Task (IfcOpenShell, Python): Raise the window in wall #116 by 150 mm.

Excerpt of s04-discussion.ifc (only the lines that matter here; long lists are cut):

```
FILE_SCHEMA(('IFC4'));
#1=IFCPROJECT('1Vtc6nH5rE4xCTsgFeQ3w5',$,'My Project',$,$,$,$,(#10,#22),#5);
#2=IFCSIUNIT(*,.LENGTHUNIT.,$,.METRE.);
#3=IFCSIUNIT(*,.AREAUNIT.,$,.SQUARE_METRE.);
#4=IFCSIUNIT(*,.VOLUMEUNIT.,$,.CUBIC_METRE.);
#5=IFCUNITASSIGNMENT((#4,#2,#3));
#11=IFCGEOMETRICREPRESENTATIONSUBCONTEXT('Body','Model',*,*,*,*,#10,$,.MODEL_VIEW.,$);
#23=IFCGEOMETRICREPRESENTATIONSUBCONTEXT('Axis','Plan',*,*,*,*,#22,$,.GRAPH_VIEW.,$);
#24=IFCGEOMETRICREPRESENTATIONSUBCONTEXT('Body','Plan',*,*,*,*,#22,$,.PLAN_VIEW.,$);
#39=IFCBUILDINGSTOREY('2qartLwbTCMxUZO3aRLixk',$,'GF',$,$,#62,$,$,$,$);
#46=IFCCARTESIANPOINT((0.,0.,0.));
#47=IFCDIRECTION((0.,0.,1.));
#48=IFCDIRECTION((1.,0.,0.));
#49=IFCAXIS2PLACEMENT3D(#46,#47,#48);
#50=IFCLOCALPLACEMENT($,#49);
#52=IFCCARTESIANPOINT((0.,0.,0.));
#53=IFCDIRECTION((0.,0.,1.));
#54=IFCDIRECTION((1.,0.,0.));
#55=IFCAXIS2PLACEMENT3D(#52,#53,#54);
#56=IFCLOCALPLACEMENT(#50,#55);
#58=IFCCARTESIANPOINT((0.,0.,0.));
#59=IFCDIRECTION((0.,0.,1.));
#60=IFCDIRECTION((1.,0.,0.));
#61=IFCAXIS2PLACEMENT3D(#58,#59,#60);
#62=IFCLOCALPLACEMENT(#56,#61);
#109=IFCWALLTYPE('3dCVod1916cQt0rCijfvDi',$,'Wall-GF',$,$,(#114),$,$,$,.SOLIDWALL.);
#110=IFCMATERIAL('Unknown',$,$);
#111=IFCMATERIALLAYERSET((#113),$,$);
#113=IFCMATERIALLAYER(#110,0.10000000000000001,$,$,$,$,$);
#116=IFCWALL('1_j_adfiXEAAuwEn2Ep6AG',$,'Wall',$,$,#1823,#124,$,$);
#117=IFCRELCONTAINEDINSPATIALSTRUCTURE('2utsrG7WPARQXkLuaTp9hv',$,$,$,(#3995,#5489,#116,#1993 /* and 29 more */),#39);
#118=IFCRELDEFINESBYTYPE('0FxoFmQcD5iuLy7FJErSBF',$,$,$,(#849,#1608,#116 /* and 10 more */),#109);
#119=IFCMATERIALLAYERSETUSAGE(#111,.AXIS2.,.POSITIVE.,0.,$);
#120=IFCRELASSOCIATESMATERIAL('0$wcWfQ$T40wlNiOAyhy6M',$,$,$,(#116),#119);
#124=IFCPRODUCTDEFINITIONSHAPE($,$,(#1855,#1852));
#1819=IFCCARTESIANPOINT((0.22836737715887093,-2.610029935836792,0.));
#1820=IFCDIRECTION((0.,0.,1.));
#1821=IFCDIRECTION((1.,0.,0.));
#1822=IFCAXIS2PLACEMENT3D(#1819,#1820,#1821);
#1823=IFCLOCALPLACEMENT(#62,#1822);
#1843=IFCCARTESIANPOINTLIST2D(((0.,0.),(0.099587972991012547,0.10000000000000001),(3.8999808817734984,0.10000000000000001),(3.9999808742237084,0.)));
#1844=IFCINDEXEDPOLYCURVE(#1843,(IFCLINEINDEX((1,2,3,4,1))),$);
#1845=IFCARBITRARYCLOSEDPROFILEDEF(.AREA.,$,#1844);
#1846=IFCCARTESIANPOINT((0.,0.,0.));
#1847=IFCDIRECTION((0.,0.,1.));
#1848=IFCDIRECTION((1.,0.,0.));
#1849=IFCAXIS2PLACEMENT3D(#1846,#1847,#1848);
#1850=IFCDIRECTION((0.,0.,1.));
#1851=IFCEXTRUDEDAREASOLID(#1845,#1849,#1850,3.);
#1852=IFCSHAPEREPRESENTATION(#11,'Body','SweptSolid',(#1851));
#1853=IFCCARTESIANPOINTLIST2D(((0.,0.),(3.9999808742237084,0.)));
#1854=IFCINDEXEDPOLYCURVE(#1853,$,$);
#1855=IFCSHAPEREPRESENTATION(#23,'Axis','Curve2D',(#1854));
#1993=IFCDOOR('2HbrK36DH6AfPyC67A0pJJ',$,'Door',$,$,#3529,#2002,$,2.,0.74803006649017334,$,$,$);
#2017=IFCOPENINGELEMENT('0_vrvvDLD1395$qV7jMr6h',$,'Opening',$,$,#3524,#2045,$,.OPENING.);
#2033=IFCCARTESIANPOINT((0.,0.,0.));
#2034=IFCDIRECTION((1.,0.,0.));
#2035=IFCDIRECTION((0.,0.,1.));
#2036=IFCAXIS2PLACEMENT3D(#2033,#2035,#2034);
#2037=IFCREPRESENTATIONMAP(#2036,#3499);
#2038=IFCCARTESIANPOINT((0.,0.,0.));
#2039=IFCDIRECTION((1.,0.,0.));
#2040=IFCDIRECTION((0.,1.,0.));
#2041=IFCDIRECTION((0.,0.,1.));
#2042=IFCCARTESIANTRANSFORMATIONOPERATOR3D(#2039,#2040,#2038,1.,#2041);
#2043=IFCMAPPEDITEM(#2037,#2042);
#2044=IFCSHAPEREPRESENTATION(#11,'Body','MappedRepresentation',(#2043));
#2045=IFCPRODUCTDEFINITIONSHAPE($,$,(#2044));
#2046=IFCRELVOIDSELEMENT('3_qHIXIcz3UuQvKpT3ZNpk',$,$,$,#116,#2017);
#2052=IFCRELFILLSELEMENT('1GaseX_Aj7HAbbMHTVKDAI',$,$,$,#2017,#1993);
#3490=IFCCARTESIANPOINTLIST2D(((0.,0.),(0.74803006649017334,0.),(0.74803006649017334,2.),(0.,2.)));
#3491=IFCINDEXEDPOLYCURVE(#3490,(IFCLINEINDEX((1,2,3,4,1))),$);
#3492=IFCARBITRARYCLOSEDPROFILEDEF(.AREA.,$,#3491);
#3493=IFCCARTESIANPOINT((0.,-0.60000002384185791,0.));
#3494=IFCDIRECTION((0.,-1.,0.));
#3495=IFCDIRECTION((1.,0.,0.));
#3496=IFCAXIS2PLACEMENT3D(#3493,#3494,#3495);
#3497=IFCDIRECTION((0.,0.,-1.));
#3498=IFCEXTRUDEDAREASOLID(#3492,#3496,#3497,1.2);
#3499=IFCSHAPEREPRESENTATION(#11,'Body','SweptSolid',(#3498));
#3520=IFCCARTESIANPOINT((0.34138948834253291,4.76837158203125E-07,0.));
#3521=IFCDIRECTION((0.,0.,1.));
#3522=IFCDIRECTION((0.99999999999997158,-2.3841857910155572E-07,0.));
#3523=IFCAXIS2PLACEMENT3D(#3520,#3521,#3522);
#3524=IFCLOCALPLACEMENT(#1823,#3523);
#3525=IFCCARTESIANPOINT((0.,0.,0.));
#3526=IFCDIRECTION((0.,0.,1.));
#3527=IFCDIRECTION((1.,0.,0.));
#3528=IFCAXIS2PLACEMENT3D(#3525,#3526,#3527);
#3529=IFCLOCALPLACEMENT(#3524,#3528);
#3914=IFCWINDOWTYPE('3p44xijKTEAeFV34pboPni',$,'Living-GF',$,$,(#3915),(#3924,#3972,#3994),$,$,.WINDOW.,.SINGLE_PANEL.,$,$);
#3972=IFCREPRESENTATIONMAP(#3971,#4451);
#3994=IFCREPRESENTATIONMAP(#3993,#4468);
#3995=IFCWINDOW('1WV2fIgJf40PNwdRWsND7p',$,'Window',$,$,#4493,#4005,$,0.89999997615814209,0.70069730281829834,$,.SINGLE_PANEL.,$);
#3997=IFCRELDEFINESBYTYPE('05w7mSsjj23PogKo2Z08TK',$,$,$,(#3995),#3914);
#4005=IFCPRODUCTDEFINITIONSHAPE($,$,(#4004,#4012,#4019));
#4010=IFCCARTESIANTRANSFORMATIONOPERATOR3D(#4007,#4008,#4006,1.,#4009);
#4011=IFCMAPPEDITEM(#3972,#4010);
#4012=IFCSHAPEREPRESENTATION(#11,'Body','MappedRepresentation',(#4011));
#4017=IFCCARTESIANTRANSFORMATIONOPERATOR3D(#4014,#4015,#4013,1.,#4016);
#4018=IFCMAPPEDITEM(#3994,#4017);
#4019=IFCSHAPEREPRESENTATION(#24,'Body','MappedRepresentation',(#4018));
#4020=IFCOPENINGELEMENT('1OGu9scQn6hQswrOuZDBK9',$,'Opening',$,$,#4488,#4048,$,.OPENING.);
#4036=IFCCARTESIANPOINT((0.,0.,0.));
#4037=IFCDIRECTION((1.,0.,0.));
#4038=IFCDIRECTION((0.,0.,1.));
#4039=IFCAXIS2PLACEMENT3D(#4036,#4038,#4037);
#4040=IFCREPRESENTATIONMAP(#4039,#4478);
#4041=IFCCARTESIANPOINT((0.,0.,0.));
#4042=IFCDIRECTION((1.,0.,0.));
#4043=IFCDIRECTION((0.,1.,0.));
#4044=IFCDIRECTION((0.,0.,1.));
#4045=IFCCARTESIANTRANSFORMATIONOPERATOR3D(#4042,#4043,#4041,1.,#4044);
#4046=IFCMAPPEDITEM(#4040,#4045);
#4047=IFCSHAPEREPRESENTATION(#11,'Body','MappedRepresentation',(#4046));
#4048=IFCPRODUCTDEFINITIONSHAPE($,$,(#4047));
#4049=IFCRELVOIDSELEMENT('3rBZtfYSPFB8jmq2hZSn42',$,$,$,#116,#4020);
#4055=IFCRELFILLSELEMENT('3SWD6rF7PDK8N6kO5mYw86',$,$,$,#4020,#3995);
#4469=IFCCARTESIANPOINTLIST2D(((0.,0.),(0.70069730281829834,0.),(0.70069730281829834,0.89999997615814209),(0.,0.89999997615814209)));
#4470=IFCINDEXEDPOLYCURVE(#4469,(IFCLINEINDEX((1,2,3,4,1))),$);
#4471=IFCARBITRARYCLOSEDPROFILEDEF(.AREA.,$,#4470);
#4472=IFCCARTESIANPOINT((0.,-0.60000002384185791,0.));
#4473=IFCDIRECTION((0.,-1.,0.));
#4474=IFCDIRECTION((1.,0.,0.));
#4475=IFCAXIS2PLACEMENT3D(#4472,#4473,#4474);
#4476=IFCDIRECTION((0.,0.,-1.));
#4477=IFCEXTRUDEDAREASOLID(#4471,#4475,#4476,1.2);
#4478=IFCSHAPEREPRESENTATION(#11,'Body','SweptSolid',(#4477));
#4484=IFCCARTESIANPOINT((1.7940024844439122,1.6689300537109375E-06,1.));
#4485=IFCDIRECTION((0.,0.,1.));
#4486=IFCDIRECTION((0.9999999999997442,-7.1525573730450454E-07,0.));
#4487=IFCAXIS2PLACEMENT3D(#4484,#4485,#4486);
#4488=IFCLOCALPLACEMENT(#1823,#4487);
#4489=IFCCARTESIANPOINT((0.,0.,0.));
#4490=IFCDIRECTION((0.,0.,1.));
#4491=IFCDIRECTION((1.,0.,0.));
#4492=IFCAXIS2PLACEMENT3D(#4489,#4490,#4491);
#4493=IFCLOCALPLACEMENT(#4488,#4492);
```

```python
import numpy as np
import ifcopenshell
import ifcopenshell.api.geometry
import ifcopenshell.util.placement
import ifcopenshell.util.unit

model = ifcopenshell.open("s04-discussion.ifc")
unit_scale = ifcopenshell.util.unit.calculate_unit_scale(model)

window = model.by_guid("1WV2fIgJf40PNwdRWsND7p")
opening = window.FillsVoids[0].RelatingOpeningElement
dz = 0.15

shift = np.array([0.0, 0.0, dz])
# The window is placed relative to its opening, so it follows when the opening moves.
matrix = ifcopenshell.util.placement.get_local_placement(opening.ObjectPlacement)
matrix[:3, 3] += shift
ifcopenshell.api.geometry.edit_object_placement(
    model, product=opening, matrix=matrix, is_si=False, should_transform_children=True
)

print(f"moved by {dz * unit_scale:+.3f} m")

model.write("s04-discussion_v2.ifc")
```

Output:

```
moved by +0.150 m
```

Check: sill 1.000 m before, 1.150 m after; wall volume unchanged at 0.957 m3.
